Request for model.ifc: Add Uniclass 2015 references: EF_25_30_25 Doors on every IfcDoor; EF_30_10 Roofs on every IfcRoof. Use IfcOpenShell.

First a look at what the model holds.

```python
import ifcopenshell

model = ifcopenshell.open("model.ifc")
print(model.schema)
print("classifications:", [c.Name for c in model.by_type("IfcClassification")])
for ifc_class in ("IfcDoor", "IfcRoof", "IfcStair", "IfcWall", "IfcWindow"):
    print(ifc_class, len(model.by_type(ifc_class)))
```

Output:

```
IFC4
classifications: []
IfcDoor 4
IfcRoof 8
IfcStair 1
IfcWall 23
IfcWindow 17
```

```python
import ifcopenshell
import ifcopenshell.api.classification

model = ifcopenshell.open("model.ifc")

system = ifcopenshell.api.classification.add_classification(model, classification="Uniclass 2015")

codes = {
    "IfcDoor": ("EF_25_30_25", "Doors"),
    "IfcRoof": ("EF_30_10", "Roofs"),
}
for ifc_class, (code, name) in codes.items():
    products = model.by_type(ifc_class)
    ifcopenshell.api.classification.add_reference(
        model, products=products, classification=system, identification=code, name=name
    )
    print(code, len(products))

model.write("model_rev.ifc")
```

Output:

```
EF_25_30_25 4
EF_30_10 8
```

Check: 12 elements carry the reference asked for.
